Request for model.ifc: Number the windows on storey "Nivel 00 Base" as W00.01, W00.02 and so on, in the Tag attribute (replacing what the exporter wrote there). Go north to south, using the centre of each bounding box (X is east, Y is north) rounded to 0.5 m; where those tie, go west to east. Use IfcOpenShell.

First a look at what the model holds.

```python
import ifcopenshell
import ifcopenshell.util.element
import ifcopenshell.util.placement

model = ifcopenshell.open("model.ifc")
print(model.schema)
storey = next(s for s in model.by_type("IfcBuildingStorey") if s.Name == "Nivel 00 Base")
windows = [e for e in ifcopenshell.util.element.get_decomposition(storey) if e.is_a("IfcWindow")]
for e in sorted(windows, key=lambda e: e.id()):
    origin = ifcopenshell.util.placement.get_local_placement(e.ObjectPlacement)[:3, 3]
    print(e.id(), e.Tag, e.Name, origin.round(2) + 0.0, sep=" | ")
```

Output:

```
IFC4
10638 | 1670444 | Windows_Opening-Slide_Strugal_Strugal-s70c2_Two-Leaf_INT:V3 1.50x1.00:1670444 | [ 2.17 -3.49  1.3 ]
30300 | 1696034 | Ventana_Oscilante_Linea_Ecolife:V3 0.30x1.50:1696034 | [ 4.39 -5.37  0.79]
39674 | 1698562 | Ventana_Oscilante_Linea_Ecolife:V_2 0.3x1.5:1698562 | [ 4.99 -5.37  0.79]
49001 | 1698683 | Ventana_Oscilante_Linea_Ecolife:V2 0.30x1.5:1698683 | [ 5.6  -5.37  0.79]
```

```python
import ifcopenshell
import ifcopenshell.geom
import ifcopenshell.util.element
import ifcopenshell.util.shape

model = ifcopenshell.open("model.ifc")
settings = ifcopenshell.geom.settings()
settings.set("use-world-coords", True)


def centre(element):
    shape = ifcopenshell.geom.create_shape(settings, element)
    return ifcopenshell.util.shape.get_bbox_centroid(shape.geometry)


storey = next(s for s in model.by_type("IfcBuildingStorey") if s.Name == "Nivel 00 Base")
windows = [e for e in ifcopenshell.util.element.get_decomposition(storey) if e.is_a("IfcWindow")]

# Insertion points can sit at a corner or the storey origin, so sort by the geometry (in metres).
centres = {e: centre(e) for e in windows}
windows.sort(key=lambda e: (-round(centres[e][1] / 0.5), centres[e][0]))

for i, e in enumerate(windows, start=1):
    number = f"W00.{i:02d}"
    e.Tag = number
    print(e.id(), number)

model.write("model_updated.ifc")
```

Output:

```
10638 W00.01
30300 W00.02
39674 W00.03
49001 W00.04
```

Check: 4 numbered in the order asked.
